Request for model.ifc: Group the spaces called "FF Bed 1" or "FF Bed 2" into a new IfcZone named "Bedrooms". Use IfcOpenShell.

First a look at what the model holds.

```python
import ifcopenshell

model = ifcopenshell.open("model.ifc")
print(model.schema)
seen = {}
for space in model.by_type("IfcSpace"):
    seen[space.Name] = seen.get(space.Name, 0) + 1
for name, count in sorted(seen.items(), key=str):
    print(count, "x", name)
print("zones:", [z.Name for z in model.by_type("IfcZone")][:20])
```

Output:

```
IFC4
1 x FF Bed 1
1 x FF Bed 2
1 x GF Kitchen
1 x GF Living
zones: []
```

```python
import ifcopenshell
import ifcopenshell.api.group
import ifcopenshell.api.root

model = ifcopenshell.open("model.ifc")

names = {"FF Bed 1", "FF Bed 2"}
spaces = [s for s in model.by_type("IfcSpace") if s.Name in names]

zone = ifcopenshell.api.root.create_entity(model, ifc_class="IfcZone", name="Bedrooms")
ifcopenshell.api.group.assign_group(model, products=spaces, group=zone)
print(len(spaces), "spaces in", zone.Name)

model.write("model_edited.ifc")
```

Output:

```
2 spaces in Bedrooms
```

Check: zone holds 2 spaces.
